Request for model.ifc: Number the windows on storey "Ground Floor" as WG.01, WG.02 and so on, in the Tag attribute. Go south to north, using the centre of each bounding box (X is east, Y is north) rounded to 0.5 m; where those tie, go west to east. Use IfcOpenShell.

First a look at what the model holds.

```python
import ifcopenshell
import ifcopenshell.util.element
import ifcopenshell.util.placement

model = ifcopenshell.open("model.ifc")
print(model.schema)
storey = next(s for s in model.by_type("IfcBuildingStorey") if s.Name == "Ground Floor")
windows = [e for e in ifcopenshell.util.element.get_decomposition(storey) if e.is_a("IfcWindow")]
for e in sorted(windows, key=lambda e: e.id()):
    origin = ifcopenshell.util.placement.get_local_placement(e.ObjectPlacement)[:3, 3]
    print(e.id(), e.Tag, e.Name, origin.round(2) + 0.0, sep=" | ")
```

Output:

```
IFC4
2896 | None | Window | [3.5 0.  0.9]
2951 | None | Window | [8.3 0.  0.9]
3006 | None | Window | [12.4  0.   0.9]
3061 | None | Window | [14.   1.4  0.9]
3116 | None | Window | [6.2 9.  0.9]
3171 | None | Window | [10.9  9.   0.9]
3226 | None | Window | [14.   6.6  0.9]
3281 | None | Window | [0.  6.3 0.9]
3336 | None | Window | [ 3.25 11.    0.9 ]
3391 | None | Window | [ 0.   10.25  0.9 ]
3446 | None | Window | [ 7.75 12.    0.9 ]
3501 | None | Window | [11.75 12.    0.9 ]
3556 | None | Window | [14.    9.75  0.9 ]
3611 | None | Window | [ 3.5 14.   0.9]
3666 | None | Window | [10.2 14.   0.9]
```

```python
import ifcopenshell
import ifcopenshell.geom
import ifcopenshell.util.element
import ifcopenshell.util.shape

model = ifcopenshell.open("model.ifc")
settings = ifcopenshell.geom.settings()
settings.set("use-world-coords", True)


def centre(element):
    shape = ifcopenshell.geom.create_shape(settings, element)
    return ifcopenshell.util.shape.get_bbox_centroid(shape.geometry)


storey = next(s for s in model.by_type("IfcBuildingStorey") if s.Name == "Ground Floor")
windows = [e for e in ifcopenshell.util.element.get_decomposition(storey) if e.is_a("IfcWindow")]

# Insertion points can sit at a corner or the storey origin, so sort by the geometry (in metres).
centres = {e: centre(e) for e in windows}
windows.sort(key=lambda e: (round(centres[e][1] / 0.5), centres[e][0]))

for i, e in enumerate(windows, start=1):
    number = f"WG.{i:02d}"
    e.Tag = number
    print(e.id(), number)

model.write("model_updated.ifc")
```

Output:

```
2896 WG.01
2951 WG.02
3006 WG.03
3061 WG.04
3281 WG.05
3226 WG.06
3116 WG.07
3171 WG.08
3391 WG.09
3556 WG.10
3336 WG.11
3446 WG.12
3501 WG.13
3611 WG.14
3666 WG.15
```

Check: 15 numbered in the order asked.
